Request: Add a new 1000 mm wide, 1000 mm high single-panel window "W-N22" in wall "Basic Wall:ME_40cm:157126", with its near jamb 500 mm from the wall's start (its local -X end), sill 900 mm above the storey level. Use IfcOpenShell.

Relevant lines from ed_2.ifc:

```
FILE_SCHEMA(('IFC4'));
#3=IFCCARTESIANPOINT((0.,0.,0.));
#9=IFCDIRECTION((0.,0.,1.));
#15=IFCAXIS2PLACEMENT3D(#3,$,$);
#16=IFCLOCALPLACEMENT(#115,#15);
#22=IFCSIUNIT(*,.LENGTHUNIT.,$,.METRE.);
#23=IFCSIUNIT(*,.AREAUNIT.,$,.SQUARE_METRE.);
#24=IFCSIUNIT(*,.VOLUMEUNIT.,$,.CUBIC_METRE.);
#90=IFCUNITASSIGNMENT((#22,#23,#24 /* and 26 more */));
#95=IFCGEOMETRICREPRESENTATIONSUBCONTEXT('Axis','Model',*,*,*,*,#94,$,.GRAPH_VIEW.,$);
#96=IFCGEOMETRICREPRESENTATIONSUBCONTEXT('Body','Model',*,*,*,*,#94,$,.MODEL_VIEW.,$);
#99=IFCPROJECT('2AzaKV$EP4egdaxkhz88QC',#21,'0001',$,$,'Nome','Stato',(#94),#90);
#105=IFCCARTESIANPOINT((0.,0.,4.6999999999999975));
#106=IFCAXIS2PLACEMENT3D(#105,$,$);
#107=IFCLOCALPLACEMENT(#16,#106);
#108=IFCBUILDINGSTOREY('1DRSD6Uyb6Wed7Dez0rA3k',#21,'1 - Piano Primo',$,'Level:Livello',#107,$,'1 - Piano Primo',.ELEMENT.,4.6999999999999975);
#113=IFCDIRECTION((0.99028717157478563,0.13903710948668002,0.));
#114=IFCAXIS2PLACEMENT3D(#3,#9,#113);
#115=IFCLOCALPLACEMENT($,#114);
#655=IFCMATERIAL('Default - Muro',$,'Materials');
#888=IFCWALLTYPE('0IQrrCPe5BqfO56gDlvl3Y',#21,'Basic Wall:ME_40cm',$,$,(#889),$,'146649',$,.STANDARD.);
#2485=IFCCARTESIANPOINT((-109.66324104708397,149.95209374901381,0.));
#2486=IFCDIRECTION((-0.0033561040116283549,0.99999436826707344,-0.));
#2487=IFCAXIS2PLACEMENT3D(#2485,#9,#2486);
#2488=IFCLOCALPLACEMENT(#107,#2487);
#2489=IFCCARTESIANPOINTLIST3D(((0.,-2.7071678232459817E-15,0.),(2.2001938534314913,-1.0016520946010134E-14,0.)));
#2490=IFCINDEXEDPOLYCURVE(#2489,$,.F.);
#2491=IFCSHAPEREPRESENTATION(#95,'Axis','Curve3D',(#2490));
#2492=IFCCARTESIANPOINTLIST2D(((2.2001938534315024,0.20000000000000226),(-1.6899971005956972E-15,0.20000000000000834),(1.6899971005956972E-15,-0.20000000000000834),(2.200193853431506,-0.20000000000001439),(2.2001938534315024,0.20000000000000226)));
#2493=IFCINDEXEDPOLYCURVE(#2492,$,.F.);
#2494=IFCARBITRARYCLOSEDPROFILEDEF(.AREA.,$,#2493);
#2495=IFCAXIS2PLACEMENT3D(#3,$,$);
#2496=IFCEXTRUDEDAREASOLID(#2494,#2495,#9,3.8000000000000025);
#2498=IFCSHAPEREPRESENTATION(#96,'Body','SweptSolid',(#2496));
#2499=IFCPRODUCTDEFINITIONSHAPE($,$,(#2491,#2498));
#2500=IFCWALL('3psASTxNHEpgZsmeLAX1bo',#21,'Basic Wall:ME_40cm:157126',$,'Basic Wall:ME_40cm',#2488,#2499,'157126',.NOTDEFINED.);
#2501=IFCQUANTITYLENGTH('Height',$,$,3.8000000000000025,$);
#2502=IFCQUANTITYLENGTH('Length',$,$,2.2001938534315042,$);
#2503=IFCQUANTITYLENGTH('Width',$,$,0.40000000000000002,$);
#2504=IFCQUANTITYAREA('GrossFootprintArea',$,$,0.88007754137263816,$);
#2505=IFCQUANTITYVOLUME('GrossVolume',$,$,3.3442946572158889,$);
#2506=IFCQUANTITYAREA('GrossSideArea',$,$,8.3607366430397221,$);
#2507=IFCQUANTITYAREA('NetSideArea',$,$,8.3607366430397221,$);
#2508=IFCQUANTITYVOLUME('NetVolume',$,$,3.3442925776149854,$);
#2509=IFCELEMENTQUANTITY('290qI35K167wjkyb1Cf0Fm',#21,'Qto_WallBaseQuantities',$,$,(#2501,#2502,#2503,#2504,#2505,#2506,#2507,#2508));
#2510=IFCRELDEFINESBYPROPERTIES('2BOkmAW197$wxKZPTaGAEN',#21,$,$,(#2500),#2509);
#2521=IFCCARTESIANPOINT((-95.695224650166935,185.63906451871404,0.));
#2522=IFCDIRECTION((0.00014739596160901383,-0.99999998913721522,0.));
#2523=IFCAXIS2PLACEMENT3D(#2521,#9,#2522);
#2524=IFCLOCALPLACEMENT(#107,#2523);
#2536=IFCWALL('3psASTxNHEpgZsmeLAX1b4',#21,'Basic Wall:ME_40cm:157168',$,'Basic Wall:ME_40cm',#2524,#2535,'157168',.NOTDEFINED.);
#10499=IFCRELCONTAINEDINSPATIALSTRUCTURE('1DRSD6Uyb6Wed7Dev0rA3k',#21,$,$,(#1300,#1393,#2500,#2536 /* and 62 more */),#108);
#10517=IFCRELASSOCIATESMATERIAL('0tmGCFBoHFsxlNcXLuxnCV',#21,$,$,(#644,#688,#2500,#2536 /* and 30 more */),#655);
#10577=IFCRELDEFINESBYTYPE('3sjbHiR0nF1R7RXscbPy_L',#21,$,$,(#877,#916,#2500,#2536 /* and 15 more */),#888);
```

```python
import numpy as np
import ifcopenshell
import ifcopenshell.api.feature
import ifcopenshell.api.geometry
import ifcopenshell.api.pset
import ifcopenshell.api.root
import ifcopenshell.api.spatial
import ifcopenshell.geom
import ifcopenshell.util.element
import ifcopenshell.util.placement
import ifcopenshell.util.representation
import ifcopenshell.util.shape
import ifcopenshell.util.unit

model = ifcopenshell.open("ed_2.ifc")
unit_scale = ifcopenshell.util.unit.calculate_unit_scale(model)
area_scale = ifcopenshell.util.unit.calculate_unit_scale(model, "AREAUNIT")
volume_scale = ifcopenshell.util.unit.calculate_unit_scale(model, "VOLUMEUNIT")
settings = ifcopenshell.geom.settings()


def volume(element):
    """Net volume in cubic metres, openings subtracted."""
    shape = ifcopenshell.geom.create_shape(settings, element)
    return ifcopenshell.util.shape.get_volume(shape.geometry)


wall = model.by_guid("3psASTxNHEpgZsmeLAX1bo")
storey = ifcopenshell.util.element.get_container(wall, ifc_class="IfcBuildingStorey")
context = ifcopenshell.util.representation.get_context(model, "Model", "Body", "MODEL_VIEW")
before = volume(wall)

width, height, from_end, sill = 1, 1, 0.5, 0.9  # metres

# The wall runs along its own X axis, and the end named is its -X end.
wall_shape = ifcopenshell.geom.create_shape(settings, wall)
x, y, z = ifcopenshell.util.shape.get_vertices(wall_shape.geometry).T
start = x.min() + from_end
face, thickness = float(y.min()), float(y.max() - y.min())
wall_matrix = ifcopenshell.util.placement.get_local_placement(wall.ObjectPlacement)
level = ifcopenshell.util.placement.get_local_placement(storey.ObjectPlacement)[2, 3]


def in_wall(x, y):
    """Placement at x, y metres in the wall's axes, at sill height."""
    matrix = wall_matrix.copy()
    matrix[:, 3] = wall_matrix @ np.array([x / unit_scale, y / unit_scale, 0.0, 1.0])
    matrix[2, 3] = level + sill / unit_scale
    return matrix


# Opening: a box that overshoots both wall faces by 50 mm.
opening = ifcopenshell.api.root.create_entity(model, ifc_class="IfcOpeningElement", predefined_type="OPENING")
box = ifcopenshell.api.geometry.add_wall_representation(
    model, context=context, length=width, height=height, thickness=thickness + 0.1
)
ifcopenshell.api.geometry.assign_representation(model, product=opening, representation=box)
ifcopenshell.api.geometry.edit_object_placement(model, product=opening, matrix=in_wall(start, face - 0.05), is_si=False)
ifcopenshell.api.feature.add_feature(model, feature=opening, element=wall)

window = ifcopenshell.api.root.create_entity(model, ifc_class="IfcWindow", name="W-N22", predefined_type="WINDOW")
window.OverallWidth, window.OverallHeight = width / unit_scale, height / unit_scale
window.PartitioningType = "SINGLE_PANEL"
body = ifcopenshell.api.geometry.add_window_representation(
    model,
    context=context,
    overall_width=window.OverallWidth,
    overall_height=window.OverallHeight,
    partition_type="SINGLE_PANEL",
)
ifcopenshell.api.geometry.assign_representation(model, product=window, representation=body)
ifcopenshell.api.spatial.assign_container(model, products=[window], relating_structure=storey)
ifcopenshell.api.feature.add_filling(model, opening=opening, element=window)

# Centre the window in the wall's thickness.
ifcopenshell.api.geometry.edit_object_placement(model, product=window, matrix=in_wall(start, face), is_si=False)
window_shape = ifcopenshell.geom.create_shape(settings, window)
depth = ifcopenshell.util.shape.get_vertices(window_shape.geometry)[:, 1]
offset = face + thickness / 2 - (depth.min() + depth.max()) / 2
ifcopenshell.api.geometry.edit_object_placement(model, product=window, matrix=in_wall(start, offset), is_si=False)

after = volume(wall)

# Update the wall's stored quantities.
qto = model.by_id(ifcopenshell.util.element.get_pset(wall, "Qto_WallBaseQuantities", should_inherit=False)["id"])
ifcopenshell.api.pset.edit_qto(model, qto=qto, properties={
    "NetSideArea": after / thickness / area_scale,
    "NetVolume": after / volume_scale,
})

print(f"wall volume {before:.3f} -> {after:.3f} m3")

model.write("ed_2-out.ifc")
```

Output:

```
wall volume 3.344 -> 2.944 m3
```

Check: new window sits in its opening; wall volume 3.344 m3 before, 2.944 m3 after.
